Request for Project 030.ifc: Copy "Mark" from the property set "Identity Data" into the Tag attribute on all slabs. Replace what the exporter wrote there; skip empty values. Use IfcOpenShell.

First a look at what the model holds.

```python
import ifcopenshell
import ifcopenshell.util.element

model = ifcopenshell.open("Project 030.ifc")
print(model.schema)
slabs = model.by_type("IfcSlab")
print(len(slabs), "slabs")
for e in slabs[:8]:
    source = ifcopenshell.util.element.get_pset(e, "Identity Data", "Mark")
    target = e.Tag
    print(e.id(), repr(source), repr(target), sep=" | ")
```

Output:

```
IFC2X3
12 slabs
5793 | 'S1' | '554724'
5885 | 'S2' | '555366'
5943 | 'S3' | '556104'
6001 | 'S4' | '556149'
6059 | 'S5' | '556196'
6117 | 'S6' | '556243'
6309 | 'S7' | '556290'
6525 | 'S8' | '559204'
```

```python
import ifcopenshell
import ifcopenshell.util.element

model = ifcopenshell.open("Project 030.ifc")

count = 0
for e in model.by_type("IfcSlab"):
    value = ifcopenshell.util.element.get_pset(e, "Identity Data", "Mark")
    current = e.Tag
    if not value or not value.strip() or current == value:
        continue
    e.Tag = value
    count += 1

print(count, "slabs updated")

model.write("Project 030_updated.ifc")
```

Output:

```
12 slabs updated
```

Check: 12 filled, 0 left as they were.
